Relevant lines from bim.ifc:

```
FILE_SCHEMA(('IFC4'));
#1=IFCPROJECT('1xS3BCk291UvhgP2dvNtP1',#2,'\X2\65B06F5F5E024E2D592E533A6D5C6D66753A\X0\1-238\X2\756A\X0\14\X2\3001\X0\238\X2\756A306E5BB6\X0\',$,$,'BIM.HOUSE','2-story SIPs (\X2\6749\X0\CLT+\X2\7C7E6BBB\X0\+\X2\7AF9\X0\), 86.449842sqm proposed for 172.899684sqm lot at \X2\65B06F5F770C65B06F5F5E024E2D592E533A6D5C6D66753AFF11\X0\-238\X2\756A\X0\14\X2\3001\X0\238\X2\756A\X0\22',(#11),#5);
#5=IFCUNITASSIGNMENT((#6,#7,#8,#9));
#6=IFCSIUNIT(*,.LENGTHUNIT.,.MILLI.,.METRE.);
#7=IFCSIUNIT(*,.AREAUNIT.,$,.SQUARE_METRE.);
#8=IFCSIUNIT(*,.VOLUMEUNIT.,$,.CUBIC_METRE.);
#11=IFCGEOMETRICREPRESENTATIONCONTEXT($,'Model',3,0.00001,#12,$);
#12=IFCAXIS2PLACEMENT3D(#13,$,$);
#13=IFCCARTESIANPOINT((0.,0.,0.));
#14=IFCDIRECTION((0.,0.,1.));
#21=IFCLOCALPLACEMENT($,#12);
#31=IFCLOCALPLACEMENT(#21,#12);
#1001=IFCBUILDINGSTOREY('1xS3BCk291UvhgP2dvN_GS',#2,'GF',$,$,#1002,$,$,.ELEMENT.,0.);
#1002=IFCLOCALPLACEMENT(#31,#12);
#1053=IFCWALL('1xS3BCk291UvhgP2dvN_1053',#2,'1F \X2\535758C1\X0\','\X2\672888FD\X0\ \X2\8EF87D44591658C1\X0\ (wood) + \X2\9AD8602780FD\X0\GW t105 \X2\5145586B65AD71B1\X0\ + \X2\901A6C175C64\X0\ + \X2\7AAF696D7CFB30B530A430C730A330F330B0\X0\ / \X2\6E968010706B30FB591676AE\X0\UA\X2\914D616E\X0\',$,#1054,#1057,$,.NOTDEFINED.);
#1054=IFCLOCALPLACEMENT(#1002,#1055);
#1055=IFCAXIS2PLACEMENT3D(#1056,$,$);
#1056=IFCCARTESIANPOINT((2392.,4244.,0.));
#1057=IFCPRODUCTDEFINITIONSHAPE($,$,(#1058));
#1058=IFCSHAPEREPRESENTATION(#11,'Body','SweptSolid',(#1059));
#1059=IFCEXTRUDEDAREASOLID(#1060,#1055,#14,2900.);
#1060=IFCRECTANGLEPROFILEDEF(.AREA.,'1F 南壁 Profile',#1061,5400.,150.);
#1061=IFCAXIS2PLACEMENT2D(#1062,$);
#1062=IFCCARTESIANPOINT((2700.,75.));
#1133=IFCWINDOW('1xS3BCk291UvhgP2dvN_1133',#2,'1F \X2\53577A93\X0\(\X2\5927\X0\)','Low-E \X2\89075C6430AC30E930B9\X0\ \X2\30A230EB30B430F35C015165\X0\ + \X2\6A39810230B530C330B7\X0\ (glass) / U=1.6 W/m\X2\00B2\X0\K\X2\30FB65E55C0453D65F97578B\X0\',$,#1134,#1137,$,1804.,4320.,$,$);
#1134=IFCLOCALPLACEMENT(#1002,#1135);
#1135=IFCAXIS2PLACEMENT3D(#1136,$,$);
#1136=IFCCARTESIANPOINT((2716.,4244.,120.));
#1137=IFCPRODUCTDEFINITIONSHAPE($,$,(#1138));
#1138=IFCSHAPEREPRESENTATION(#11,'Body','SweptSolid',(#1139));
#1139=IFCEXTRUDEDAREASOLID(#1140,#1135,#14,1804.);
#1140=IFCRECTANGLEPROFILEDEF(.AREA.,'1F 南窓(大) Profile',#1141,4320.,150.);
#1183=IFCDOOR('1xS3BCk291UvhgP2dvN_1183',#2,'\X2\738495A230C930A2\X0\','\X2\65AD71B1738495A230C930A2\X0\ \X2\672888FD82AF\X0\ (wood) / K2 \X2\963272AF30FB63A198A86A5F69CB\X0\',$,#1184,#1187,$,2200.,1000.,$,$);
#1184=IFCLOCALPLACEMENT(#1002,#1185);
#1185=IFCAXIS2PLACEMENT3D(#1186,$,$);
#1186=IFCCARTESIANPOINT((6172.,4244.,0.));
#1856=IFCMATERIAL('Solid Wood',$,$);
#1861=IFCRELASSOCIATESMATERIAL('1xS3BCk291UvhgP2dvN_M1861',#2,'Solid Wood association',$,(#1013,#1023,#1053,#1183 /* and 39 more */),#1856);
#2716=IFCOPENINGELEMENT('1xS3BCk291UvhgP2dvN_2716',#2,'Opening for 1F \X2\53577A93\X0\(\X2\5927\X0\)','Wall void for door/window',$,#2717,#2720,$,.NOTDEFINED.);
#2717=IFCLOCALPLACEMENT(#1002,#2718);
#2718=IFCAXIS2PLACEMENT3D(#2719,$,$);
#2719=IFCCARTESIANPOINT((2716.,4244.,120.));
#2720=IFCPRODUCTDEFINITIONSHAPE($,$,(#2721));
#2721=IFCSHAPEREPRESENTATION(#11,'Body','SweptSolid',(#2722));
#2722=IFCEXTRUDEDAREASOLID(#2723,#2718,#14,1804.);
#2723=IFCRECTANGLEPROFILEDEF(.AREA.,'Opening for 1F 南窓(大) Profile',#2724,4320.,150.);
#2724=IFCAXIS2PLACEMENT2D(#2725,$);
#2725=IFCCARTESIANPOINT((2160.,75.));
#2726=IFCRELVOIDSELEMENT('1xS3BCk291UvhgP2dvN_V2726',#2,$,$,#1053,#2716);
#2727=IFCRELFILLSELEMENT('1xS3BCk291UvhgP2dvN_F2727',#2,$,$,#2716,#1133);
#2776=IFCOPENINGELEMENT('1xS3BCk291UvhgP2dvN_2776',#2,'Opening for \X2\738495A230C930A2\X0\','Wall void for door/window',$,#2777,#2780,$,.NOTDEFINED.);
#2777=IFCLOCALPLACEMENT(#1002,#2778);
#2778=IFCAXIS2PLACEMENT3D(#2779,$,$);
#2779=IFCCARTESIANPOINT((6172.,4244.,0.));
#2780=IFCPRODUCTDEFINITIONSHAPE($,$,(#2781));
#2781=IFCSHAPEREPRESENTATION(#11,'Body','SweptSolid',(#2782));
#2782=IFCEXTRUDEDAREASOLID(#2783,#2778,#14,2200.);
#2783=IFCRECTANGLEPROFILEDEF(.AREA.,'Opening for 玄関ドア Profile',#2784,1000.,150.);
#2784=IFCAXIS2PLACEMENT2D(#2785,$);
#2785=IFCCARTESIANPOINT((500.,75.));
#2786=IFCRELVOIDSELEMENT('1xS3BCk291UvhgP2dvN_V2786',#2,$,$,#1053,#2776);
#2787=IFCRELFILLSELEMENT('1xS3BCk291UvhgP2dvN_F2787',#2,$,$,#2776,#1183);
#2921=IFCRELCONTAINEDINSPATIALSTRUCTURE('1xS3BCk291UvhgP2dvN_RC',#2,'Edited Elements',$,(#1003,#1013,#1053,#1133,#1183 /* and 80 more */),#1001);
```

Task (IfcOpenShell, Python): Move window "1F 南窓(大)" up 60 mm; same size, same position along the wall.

```python
import numpy as np
import ifcopenshell
import ifcopenshell.api.geometry
import ifcopenshell.util.placement
import ifcopenshell.util.unit

model = ifcopenshell.open("bim.ifc")
unit_scale = ifcopenshell.util.unit.calculate_unit_scale(model)

window = model.by_guid("1xS3BCk291UvhgP2dvN_1133")
opening = window.FillsVoids[0].RelatingOpeningElement
dz = 0.06 / unit_scale

shift = np.array([0.0, 0.0, dz])
# The window is not placed relative to its opening, so move both.
for product in (opening, window):
    matrix = ifcopenshell.util.placement.get_local_placement(product.ObjectPlacement)
    matrix[:3, 3] += shift
    ifcopenshell.api.geometry.edit_object_placement(model, product=product, matrix=matrix, is_si=False)

print(f"moved by {dz * unit_scale:+.3f} m")

model.write("bim_rev.ifc")
```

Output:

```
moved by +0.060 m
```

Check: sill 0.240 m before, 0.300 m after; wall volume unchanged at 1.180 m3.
